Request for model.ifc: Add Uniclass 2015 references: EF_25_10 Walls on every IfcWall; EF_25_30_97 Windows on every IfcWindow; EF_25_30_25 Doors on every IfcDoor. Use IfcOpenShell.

First a look at what the model holds.

```python
import ifcopenshell

model = ifcopenshell.open("model.ifc")
print(model.schema)
print("classifications:", [c.Name for c in model.by_type("IfcClassification")])
for ifc_class in ("IfcDoor", "IfcRoof", "IfcStair", "IfcWall", "IfcWindow"):
    print(ifc_class, len(model.by_type(ifc_class)))
```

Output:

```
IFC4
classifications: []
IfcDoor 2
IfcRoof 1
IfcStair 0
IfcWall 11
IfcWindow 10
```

```python
import ifcopenshell
import ifcopenshell.api.classification

model = ifcopenshell.open("model.ifc")

system = ifcopenshell.api.classification.add_classification(model, classification="Uniclass 2015")

codes = {
    "IfcWall": ("EF_25_10", "Walls"),
    "IfcWindow": ("EF_25_30_97", "Windows"),
    "IfcDoor": ("EF_25_30_25", "Doors"),
}
for ifc_class, (code, name) in codes.items():
    products = model.by_type(ifc_class)
    ifcopenshell.api.classification.add_reference(
        model, products=products, classification=system, identification=code, name=name
    )
    print(code, len(products))

model.write("model_rev.ifc")
```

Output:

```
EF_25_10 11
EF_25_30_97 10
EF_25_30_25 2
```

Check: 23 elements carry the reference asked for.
